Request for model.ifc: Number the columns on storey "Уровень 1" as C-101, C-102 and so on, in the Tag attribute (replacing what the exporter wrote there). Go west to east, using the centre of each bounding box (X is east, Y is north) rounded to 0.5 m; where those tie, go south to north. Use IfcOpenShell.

First a look at what the model holds.

```python
import ifcopenshell
import ifcopenshell.util.element
import ifcopenshell.util.placement

model = ifcopenshell.open("model.ifc")
print(model.schema)
storey = next(s for s in model.by_type("IfcBuildingStorey") if s.Name == "Уровень 1")
columns = [e for e in ifcopenshell.util.element.get_decomposition(storey) if e.is_a("IfcColumn")]
for e in sorted(columns, key=lambda e: e.id()):
    origin = ifcopenshell.util.placement.get_local_placement(e.ObjectPlacement)[:3, 3]
    print(e.id(), e.Tag, e.Name, origin.round(2) + 0.0, sep=" | ")
```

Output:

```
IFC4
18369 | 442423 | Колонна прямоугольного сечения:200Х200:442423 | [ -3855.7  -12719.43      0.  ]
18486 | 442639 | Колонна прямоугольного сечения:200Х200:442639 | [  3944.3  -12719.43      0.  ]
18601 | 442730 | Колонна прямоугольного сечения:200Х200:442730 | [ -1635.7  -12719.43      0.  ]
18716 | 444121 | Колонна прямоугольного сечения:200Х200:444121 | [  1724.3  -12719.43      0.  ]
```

```python
import ifcopenshell
import ifcopenshell.geom
import ifcopenshell.util.element
import ifcopenshell.util.shape

model = ifcopenshell.open("model.ifc")
settings = ifcopenshell.geom.settings()
settings.set("use-world-coords", True)


def centre(element):
    shape = ifcopenshell.geom.create_shape(settings, element)
    return ifcopenshell.util.shape.get_bbox_centroid(shape.geometry)


storey = next(s for s in model.by_type("IfcBuildingStorey") if s.Name == "Уровень 1")
columns = [e for e in ifcopenshell.util.element.get_decomposition(storey) if e.is_a("IfcColumn")]

# Insertion points can sit at a corner or the storey origin, so sort by the geometry (in metres).
centres = {e: centre(e) for e in columns}
columns.sort(key=lambda e: (round(centres[e][0] / 0.5), centres[e][1]))

for i, e in enumerate(columns, start=1):
    number = f"C-1{i:02d}"
    e.Tag = number
    print(e.id(), number)

model.write("model_edited.ifc")
```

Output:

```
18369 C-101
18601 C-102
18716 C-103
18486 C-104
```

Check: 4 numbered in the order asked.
